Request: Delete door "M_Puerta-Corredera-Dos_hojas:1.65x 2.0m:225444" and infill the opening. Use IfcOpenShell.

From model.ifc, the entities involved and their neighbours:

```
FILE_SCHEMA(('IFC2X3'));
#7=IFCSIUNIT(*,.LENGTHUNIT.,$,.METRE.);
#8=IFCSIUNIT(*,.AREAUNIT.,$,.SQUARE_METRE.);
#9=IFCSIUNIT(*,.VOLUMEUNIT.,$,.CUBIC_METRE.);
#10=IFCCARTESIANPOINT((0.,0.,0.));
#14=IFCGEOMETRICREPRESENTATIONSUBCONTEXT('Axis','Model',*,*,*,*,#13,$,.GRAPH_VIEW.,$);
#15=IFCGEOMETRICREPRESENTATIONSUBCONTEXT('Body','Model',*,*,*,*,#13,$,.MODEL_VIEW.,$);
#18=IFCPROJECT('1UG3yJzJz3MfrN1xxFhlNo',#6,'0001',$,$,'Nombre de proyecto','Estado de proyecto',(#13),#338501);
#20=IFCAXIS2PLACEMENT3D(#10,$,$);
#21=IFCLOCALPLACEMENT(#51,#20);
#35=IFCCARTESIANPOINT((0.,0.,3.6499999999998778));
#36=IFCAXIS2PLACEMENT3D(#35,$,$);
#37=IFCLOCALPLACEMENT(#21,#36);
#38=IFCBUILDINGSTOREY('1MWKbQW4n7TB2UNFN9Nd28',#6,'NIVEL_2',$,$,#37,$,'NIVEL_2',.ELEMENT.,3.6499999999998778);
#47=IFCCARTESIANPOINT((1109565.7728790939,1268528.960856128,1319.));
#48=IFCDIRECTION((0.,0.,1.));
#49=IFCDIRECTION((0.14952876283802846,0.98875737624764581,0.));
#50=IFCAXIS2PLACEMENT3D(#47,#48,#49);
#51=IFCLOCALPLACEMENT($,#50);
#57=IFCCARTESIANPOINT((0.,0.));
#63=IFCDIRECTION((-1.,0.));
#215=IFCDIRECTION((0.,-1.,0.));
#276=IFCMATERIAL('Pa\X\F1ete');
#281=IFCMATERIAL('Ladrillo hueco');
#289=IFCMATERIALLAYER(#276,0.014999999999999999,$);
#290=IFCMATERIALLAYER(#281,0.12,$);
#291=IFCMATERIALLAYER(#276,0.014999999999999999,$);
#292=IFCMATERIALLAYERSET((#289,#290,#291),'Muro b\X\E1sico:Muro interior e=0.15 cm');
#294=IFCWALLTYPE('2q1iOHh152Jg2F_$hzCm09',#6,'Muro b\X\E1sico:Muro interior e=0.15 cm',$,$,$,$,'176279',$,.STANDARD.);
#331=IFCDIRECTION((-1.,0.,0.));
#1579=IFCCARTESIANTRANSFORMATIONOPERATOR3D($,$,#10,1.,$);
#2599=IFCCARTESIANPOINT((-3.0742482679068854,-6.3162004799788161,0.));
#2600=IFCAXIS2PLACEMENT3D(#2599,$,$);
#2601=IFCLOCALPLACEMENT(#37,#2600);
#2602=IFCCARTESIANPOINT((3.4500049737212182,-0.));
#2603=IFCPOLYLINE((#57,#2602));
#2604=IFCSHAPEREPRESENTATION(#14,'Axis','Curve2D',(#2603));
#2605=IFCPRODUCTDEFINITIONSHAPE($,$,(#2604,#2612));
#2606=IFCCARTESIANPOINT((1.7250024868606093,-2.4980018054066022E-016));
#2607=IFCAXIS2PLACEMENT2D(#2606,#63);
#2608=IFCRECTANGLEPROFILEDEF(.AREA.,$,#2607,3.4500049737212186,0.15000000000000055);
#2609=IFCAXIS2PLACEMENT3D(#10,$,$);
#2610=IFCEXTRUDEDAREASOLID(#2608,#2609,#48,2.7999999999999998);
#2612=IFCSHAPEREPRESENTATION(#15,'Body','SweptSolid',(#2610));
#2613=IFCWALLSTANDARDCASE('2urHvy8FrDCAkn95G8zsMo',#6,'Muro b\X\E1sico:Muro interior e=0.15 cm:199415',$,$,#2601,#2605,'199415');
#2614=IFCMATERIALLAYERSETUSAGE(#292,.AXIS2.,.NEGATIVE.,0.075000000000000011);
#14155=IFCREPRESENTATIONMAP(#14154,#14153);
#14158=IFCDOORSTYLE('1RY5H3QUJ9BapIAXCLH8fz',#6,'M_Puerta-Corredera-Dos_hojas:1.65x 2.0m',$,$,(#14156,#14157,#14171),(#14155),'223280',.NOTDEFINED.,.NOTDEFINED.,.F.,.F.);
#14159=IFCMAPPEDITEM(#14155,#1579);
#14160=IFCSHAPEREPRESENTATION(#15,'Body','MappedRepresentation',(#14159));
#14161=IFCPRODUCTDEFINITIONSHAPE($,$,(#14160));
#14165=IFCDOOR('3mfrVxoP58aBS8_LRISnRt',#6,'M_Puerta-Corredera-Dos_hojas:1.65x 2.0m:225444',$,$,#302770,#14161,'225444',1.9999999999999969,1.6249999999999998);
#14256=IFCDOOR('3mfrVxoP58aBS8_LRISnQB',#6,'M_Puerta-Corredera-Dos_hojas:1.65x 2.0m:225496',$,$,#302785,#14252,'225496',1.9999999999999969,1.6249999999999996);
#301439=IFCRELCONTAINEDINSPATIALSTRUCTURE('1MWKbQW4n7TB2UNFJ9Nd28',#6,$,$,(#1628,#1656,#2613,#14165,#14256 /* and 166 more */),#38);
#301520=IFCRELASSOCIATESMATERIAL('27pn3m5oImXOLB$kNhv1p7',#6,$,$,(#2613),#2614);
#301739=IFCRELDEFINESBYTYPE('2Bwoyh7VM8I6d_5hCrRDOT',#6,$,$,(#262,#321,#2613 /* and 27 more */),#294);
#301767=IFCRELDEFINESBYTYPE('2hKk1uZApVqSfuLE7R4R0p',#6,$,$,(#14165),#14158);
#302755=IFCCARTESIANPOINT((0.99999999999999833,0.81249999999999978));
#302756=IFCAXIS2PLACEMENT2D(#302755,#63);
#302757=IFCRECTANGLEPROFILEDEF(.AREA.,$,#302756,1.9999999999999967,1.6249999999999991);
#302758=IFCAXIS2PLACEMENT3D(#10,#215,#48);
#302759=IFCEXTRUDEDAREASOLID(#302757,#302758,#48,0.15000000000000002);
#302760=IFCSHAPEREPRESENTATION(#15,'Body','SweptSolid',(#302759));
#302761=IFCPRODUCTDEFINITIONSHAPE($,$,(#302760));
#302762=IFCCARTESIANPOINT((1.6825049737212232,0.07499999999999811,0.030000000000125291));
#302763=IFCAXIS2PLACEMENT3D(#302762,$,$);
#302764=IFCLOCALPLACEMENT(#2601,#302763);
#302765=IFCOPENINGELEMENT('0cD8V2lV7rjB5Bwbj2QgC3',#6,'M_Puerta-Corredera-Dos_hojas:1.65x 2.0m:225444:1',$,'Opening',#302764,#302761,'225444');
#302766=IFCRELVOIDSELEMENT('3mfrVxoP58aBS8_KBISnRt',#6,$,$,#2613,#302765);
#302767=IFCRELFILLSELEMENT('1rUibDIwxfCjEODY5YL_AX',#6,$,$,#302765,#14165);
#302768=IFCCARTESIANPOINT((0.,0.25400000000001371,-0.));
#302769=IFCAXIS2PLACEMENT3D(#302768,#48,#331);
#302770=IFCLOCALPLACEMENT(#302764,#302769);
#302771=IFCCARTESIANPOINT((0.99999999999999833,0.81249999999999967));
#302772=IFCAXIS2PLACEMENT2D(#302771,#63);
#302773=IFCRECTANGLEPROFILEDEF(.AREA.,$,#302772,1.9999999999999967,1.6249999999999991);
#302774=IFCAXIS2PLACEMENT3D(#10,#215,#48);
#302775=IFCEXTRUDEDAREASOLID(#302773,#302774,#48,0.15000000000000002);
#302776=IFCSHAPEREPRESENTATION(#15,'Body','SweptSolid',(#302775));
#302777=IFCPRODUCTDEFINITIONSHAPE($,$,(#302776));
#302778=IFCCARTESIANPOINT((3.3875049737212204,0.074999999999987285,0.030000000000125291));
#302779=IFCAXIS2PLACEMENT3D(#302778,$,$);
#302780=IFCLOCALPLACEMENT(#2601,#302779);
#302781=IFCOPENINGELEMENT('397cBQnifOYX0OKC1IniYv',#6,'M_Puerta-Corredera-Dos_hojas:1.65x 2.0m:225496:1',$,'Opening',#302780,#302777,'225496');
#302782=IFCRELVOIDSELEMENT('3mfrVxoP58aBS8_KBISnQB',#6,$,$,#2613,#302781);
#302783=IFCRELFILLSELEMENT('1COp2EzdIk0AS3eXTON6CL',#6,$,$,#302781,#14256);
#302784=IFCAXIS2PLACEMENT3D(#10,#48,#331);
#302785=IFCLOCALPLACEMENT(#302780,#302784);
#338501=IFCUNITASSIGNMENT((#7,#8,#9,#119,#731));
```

```python
import ifcopenshell
import ifcopenshell.api.feature
import ifcopenshell.api.root
import ifcopenshell.geom
import ifcopenshell.util.shape

model = ifcopenshell.open("model.ifc")
settings = ifcopenshell.geom.settings()


def volume(element):
    """Net volume in cubic metres, openings subtracted."""
    shape = ifcopenshell.geom.create_shape(settings, element)
    return ifcopenshell.util.shape.get_volume(shape.geometry)


door = model.by_guid("3mfrVxoP58aBS8_LRISnRt")
opening = door.FillsVoids[0].RelatingOpeningElement
wall = opening.VoidsElements[0].RelatingBuildingElement
before = volume(wall)

ifcopenshell.api.root.remove_product(model, product=door)
ifcopenshell.api.feature.remove_feature(model, feature=opening)

after = volume(wall)

print(f"wall volume {before:.3f} -> {after:.3f} m3")

model.write("model_updated.ifc")
```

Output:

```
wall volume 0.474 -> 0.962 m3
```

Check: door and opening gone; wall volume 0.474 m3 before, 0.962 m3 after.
